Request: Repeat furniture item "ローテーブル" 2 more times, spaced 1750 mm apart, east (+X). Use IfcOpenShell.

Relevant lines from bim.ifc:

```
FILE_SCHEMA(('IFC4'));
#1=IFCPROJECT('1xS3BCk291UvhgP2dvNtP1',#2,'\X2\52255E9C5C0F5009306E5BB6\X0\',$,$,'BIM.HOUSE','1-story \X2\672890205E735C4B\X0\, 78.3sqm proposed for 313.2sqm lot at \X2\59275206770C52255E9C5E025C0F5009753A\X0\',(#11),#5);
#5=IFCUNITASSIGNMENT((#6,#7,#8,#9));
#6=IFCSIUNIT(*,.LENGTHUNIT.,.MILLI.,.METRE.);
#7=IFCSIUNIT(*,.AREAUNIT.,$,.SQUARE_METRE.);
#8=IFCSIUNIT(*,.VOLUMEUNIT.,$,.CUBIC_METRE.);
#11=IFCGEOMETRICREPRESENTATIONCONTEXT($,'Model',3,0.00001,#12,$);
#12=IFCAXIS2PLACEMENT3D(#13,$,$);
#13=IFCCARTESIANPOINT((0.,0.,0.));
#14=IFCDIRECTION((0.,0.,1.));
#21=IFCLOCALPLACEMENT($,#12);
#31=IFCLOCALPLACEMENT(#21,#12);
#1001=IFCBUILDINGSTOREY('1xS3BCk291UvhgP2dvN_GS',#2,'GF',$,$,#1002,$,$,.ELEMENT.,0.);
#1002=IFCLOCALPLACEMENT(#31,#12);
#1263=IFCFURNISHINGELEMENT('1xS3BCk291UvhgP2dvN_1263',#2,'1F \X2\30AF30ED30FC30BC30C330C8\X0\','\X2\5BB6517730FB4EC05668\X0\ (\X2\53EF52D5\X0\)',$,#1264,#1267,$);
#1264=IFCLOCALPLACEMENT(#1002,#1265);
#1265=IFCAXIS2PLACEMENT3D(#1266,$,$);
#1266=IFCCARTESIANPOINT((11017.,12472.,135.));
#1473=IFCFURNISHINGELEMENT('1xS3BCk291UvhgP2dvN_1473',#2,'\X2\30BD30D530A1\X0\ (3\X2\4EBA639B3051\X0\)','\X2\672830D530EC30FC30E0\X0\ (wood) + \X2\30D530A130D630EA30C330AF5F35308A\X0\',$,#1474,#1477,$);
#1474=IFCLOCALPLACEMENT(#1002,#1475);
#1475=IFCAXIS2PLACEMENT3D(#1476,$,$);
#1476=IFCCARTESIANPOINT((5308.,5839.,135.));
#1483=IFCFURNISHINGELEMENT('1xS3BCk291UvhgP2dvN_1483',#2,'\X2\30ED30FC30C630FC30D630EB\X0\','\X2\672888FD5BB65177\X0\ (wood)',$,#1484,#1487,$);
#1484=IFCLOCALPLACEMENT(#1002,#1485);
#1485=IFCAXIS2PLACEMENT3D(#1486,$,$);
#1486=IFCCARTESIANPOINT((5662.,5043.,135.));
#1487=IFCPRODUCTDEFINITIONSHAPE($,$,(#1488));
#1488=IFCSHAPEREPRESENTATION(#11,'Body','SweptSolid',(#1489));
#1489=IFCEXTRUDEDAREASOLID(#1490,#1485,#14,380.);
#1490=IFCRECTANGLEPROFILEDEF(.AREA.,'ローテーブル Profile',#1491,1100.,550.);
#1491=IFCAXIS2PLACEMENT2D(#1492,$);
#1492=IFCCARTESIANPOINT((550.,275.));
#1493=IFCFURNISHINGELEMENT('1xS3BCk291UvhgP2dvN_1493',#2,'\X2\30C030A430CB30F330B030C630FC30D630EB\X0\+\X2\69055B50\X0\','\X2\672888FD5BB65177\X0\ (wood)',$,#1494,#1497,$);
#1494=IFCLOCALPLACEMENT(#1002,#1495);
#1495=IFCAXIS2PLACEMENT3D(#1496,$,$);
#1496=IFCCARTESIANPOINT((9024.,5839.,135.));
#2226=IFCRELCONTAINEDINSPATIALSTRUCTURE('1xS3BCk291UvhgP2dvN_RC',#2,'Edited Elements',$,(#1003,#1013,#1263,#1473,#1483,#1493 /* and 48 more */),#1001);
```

```python
import numpy as np
import ifcopenshell
import ifcopenshell.api.geometry
import ifcopenshell.api.root
import ifcopenshell.util.element
import ifcopenshell.util.placement

model = ifcopenshell.open("bim.ifc")


def reuse_history(source, copy):
    """copy_class also copies each property set's owner history, people and application; keep the originals."""
    for rel in copy.IsDefinedBy:
        if rel.is_a("IfcRelDefinesByProperties") and (history := rel.RelatingPropertyDefinition.OwnerHistory):
            rel.RelatingPropertyDefinition.OwnerHistory = source.OwnerHistory
            ifcopenshell.util.element.remove_deep2(model, history)


source = model.by_guid("1xS3BCk291UvhgP2dvN_1483")
base = ifcopenshell.util.placement.get_local_placement(source.ObjectPlacement)
step = np.array([1.0, 0.0, 0.0]) * 1750.0

for i in range(1, 3):
    copy = ifcopenshell.api.root.copy_class(model, product=source)
    copy.Representation = ifcopenshell.util.element.copy_deep(
        model, source.Representation, exclude=["IfcGeometricRepresentationContext", "IfcRepresentationMap"]
    )
    reuse_history(source, copy)
    matrix = base.copy()
    matrix[:3, 3] += i * step
    print("added at", matrix[:3, 3].round(3) + 0.0)
    ifcopenshell.api.geometry.edit_object_placement(model, product=copy, matrix=matrix, is_si=False)

model.write("bim-out.ifc")
```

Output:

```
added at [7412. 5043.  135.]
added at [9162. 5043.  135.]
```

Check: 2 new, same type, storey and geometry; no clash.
